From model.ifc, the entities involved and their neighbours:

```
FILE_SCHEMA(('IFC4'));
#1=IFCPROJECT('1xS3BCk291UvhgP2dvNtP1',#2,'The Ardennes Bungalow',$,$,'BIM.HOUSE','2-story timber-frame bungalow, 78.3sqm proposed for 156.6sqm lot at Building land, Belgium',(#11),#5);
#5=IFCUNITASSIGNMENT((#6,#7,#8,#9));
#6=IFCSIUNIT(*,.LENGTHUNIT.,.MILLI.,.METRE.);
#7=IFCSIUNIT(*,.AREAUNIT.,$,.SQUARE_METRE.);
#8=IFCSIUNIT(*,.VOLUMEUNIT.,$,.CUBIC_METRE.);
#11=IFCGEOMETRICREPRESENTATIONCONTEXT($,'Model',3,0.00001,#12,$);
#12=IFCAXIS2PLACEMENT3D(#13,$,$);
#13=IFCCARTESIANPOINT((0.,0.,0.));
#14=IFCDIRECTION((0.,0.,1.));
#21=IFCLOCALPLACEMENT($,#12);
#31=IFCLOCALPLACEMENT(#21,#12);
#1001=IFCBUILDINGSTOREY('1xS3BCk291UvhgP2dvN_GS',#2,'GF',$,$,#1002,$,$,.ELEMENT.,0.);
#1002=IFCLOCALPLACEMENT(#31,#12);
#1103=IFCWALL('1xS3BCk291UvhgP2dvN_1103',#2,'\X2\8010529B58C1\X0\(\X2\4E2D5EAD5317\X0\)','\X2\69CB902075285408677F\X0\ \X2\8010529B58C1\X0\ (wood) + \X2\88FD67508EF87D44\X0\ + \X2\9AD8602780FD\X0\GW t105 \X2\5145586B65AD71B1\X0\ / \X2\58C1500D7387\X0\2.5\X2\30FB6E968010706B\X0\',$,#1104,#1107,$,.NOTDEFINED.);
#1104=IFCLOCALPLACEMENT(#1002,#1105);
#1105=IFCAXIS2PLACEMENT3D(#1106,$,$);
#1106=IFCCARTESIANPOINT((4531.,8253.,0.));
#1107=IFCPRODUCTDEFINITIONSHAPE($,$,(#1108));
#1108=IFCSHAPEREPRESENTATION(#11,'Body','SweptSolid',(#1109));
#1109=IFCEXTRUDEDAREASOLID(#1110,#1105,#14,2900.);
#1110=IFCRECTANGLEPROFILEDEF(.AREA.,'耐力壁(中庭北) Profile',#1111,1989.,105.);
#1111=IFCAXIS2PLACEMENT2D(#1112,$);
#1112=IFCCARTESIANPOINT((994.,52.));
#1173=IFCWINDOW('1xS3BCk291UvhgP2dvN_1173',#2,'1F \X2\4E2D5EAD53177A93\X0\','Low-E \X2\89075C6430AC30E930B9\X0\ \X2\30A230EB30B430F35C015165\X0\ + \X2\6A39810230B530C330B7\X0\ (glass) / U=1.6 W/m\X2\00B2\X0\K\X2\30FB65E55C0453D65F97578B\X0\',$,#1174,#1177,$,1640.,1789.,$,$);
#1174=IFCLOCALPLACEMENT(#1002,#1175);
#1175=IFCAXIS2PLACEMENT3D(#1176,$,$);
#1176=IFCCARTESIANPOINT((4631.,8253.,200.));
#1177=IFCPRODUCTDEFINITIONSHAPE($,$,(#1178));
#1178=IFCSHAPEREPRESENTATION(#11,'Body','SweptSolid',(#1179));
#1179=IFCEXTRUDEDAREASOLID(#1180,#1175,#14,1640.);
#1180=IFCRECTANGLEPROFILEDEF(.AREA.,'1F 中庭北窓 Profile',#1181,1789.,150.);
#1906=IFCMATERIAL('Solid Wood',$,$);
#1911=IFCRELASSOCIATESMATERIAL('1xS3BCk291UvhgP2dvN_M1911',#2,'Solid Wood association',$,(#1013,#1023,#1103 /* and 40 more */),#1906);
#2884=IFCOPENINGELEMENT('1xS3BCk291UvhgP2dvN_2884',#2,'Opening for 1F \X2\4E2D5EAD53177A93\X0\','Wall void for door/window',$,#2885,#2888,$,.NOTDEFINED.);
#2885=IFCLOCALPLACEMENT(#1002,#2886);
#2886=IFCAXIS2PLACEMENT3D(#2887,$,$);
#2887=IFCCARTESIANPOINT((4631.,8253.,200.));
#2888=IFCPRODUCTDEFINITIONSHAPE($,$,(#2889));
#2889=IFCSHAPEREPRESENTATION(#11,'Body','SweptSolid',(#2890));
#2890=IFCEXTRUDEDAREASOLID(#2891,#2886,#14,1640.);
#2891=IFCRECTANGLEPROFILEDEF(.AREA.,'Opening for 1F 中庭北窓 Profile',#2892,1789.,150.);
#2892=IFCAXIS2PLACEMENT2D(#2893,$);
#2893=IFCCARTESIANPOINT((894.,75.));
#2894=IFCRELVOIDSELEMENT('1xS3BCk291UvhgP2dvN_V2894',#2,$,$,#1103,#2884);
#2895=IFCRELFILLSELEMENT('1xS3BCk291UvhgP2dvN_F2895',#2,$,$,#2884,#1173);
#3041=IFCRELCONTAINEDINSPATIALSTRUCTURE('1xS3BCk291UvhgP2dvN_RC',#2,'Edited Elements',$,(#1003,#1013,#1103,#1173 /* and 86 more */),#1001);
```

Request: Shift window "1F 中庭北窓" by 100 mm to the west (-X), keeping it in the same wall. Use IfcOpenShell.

```python
import ifcopenshell
import ifcopenshell.api.geometry
import ifcopenshell.util.placement

model = ifcopenshell.open("model.ifc")

window = model.by_id(1173)
opening = window.FillsVoids[0].RelatingOpeningElement
wall = opening.VoidsElements[0].RelatingBuildingElement

wall_matrix = ifcopenshell.util.placement.get_local_placement(wall.ObjectPlacement)
shift = wall_matrix[:3, 0] * -100.0
before = ifcopenshell.util.placement.get_local_placement(window.ObjectPlacement)[:3, 3].copy()

# The window is not placed relative to its opening, so move both.
for product in (opening, window):
    matrix = ifcopenshell.util.placement.get_local_placement(product.ObjectPlacement)
    matrix[:3, 3] += shift
    ifcopenshell.api.geometry.edit_object_placement(model, product=product, matrix=matrix, is_si=False)

after = ifcopenshell.util.placement.get_local_placement(window.ObjectPlacement)[:3, 3]
print("window moved by", (after - before).round(3) + 0.0)

model.write("model-out.ifc")
```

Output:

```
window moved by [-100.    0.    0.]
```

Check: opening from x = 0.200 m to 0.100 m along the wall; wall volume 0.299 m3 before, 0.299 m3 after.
